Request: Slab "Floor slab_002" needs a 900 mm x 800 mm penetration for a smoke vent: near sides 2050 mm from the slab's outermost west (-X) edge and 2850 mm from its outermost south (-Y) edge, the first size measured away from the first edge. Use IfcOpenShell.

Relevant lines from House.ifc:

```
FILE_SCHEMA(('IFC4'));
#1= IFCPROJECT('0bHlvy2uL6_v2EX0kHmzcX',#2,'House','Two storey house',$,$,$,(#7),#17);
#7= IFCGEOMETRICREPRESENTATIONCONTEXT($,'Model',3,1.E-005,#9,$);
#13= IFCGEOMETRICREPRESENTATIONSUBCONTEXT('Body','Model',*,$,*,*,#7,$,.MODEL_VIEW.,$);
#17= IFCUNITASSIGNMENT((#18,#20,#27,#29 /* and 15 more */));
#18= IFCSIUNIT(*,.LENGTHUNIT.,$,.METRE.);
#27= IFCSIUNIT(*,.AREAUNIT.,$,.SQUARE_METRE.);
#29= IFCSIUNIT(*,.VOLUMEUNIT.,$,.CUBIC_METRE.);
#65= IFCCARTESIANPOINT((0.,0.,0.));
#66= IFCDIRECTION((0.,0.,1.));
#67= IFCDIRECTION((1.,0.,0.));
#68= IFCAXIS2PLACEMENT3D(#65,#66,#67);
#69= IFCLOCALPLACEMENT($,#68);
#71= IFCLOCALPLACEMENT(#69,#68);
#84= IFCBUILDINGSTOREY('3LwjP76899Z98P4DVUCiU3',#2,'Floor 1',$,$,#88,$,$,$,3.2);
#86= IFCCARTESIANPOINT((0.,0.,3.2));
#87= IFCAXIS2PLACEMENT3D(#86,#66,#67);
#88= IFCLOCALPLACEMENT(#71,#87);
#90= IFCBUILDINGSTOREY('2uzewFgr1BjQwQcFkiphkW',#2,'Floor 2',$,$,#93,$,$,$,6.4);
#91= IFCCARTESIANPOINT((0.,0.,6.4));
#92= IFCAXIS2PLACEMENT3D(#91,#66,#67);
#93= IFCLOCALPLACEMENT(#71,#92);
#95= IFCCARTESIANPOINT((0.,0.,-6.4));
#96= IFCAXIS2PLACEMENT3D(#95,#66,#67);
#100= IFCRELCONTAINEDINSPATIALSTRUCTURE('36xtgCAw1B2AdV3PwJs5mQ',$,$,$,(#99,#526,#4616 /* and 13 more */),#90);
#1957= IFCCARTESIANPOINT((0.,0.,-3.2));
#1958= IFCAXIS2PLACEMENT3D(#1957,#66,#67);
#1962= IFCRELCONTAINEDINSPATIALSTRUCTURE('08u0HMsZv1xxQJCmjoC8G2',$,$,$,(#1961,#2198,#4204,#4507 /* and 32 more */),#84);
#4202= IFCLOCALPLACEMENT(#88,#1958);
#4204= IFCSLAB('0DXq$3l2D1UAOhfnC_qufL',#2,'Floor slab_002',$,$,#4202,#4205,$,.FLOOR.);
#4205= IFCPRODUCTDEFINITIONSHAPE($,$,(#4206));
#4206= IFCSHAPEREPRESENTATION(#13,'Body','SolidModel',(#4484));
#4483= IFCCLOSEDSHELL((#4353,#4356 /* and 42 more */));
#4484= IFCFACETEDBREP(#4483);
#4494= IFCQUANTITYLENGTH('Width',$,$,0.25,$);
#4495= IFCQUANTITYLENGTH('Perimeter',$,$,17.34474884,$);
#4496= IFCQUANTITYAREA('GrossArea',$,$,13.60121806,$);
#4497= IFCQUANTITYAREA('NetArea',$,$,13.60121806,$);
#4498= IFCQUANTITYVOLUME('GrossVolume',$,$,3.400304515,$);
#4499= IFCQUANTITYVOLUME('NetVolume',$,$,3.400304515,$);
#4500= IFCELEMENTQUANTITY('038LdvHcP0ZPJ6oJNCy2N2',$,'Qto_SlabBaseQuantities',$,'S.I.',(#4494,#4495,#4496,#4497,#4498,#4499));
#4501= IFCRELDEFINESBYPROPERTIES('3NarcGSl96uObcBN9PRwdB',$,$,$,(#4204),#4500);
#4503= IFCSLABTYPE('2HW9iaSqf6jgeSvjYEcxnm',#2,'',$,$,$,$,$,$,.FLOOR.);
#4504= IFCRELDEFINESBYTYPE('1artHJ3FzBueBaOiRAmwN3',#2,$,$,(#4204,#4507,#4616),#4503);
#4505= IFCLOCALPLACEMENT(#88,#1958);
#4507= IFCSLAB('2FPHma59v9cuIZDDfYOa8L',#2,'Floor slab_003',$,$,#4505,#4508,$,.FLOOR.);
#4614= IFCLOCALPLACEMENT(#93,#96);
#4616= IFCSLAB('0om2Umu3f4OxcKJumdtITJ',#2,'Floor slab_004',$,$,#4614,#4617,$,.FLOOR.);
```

```python
import numpy as np
import ifcopenshell
import ifcopenshell.api.feature
import ifcopenshell.api.geometry
import ifcopenshell.api.pset
import ifcopenshell.api.root
import ifcopenshell.geom
import ifcopenshell.util.element
import ifcopenshell.util.placement
import ifcopenshell.util.representation
import ifcopenshell.util.shape
import ifcopenshell.util.unit

model = ifcopenshell.open("House.ifc")
unit_scale = ifcopenshell.util.unit.calculate_unit_scale(model)
area_scale = ifcopenshell.util.unit.calculate_unit_scale(model, "AREAUNIT")
volume_scale = ifcopenshell.util.unit.calculate_unit_scale(model, "VOLUMEUNIT")
settings = ifcopenshell.geom.settings()


def volume(element):
    """Net volume in cubic metres, openings subtracted."""
    shape = ifcopenshell.geom.create_shape(settings, element)
    return ifcopenshell.util.shape.get_volume(shape.geometry)


slab = model.by_guid("0DXq$3l2D1UAOhfnC_qufL")
before = volume(slab)

# Extent in the slab's own axes, in metres. The edges named are its -X and -Y sides.
slab_shape = ifcopenshell.geom.create_shape(settings, slab)
vertices = ifcopenshell.util.shape.get_vertices(slab_shape.geometry)
x_min, y_min, bottom = vertices.min(axis=0)
top = vertices[:, 2].max()

opening = ifcopenshell.api.root.create_entity(model, ifc_class="IfcOpeningElement", name="Smoke vent opening", predefined_type="OPENING")
context = ifcopenshell.util.representation.get_context(model, "Model", "Body", "MODEL_VIEW")
width, depth = 0.9, 0.8
outline = [(0.0, 0.0), (width, 0.0), (width, depth), (0.0, depth), (0.0, 0.0)]
# Overshoot both faces by 50 mm so the cut is clean.
shape = ifcopenshell.api.geometry.add_slab_representation(
    model, context=context, depth=top - bottom + 0.1, polyline=outline
)
ifcopenshell.api.geometry.assign_representation(model, product=opening, representation=shape)

matrix = ifcopenshell.util.placement.get_local_placement(slab.ObjectPlacement)
matrix[:, 3] = matrix @ np.append(np.array([x_min + 2.05, y_min + 2.85, bottom - 0.05]) / unit_scale, 1.0)
ifcopenshell.api.geometry.edit_object_placement(model, product=opening, matrix=matrix, is_si=False)
ifcopenshell.api.feature.add_feature(model, feature=opening, element=slab)

after = volume(slab)

# Update the slab's stored quantities.
qto = model.by_id(ifcopenshell.util.element.get_pset(slab, "Qto_SlabBaseQuantities", should_inherit=False)["id"])
ifcopenshell.api.pset.edit_qto(model, qto=qto, properties={
    "NetArea": after / (top - bottom) / area_scale,
    "NetVolume": after / volume_scale,
})

print(f"slab volume {before:.3f} -> {after:.3f} m3")

model.write("House_rev.ifc")
```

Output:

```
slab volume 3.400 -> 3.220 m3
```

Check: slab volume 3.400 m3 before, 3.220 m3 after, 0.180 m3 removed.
